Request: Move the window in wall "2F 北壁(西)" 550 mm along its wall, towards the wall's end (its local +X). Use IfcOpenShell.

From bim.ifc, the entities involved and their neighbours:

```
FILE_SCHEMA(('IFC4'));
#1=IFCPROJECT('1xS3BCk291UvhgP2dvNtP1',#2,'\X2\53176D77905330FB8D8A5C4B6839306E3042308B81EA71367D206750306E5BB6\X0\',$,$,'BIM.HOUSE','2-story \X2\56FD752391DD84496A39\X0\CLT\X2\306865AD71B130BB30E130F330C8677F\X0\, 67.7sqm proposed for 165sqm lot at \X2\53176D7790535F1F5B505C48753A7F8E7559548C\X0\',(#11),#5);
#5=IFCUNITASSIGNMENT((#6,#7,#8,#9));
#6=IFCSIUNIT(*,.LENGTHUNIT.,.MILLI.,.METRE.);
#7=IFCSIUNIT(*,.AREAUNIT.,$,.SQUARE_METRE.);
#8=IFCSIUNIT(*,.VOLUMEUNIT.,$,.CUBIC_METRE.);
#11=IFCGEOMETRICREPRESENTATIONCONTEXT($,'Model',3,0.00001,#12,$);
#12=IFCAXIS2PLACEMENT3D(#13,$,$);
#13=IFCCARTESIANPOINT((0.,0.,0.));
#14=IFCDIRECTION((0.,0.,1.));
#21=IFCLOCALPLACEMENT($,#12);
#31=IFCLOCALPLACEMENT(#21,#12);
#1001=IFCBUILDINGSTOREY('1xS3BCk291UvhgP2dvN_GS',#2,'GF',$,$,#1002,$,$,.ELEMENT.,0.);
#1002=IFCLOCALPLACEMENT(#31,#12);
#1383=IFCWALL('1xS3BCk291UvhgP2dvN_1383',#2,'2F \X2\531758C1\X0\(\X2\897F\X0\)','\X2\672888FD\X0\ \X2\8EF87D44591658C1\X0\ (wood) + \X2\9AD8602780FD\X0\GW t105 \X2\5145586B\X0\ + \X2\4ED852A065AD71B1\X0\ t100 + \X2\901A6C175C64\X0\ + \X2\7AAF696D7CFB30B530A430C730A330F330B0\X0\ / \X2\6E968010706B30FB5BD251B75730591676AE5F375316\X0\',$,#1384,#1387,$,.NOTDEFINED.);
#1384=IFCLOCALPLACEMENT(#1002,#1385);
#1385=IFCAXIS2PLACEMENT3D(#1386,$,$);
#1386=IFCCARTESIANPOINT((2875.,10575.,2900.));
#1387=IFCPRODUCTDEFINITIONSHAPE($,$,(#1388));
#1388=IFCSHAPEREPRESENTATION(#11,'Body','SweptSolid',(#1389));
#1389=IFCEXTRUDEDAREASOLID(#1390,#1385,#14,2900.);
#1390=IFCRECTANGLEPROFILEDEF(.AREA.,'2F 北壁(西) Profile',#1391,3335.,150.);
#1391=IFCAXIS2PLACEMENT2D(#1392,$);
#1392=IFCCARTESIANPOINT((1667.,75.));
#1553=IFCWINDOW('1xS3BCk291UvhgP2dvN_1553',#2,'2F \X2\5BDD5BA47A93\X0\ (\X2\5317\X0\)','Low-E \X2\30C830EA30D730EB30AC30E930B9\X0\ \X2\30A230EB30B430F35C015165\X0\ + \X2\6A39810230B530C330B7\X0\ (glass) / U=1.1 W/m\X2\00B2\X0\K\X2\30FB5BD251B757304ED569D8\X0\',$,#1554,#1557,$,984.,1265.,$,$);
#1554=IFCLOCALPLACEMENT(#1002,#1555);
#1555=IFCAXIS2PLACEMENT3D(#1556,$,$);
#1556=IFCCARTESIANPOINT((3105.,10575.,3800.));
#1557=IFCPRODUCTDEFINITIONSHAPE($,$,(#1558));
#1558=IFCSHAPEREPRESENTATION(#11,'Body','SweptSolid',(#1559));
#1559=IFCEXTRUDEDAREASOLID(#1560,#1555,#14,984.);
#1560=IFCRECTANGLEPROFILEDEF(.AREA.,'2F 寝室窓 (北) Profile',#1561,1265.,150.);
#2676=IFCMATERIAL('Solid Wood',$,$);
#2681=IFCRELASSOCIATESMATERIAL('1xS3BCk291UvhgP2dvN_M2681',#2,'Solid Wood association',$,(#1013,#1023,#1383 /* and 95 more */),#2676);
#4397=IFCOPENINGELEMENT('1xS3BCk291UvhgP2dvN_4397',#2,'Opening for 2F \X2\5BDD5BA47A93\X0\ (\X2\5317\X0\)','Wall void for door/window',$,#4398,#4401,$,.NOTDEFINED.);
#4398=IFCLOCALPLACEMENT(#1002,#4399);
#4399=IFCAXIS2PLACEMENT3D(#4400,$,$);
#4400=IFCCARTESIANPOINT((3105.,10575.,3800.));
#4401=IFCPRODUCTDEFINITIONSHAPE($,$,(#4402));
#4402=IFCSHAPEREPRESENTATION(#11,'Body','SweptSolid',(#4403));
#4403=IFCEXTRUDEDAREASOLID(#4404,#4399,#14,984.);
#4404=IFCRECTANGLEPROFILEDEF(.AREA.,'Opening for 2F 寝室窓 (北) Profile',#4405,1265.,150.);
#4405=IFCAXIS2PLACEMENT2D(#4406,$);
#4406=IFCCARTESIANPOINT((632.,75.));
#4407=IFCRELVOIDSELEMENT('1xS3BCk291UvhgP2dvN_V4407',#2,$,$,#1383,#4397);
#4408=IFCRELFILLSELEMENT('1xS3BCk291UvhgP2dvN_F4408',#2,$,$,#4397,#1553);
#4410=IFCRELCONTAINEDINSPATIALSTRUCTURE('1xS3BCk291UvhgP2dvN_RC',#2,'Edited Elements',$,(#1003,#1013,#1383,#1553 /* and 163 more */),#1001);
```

```python
import ifcopenshell
import ifcopenshell.api.geometry
import ifcopenshell.util.placement
import ifcopenshell.util.unit

model = ifcopenshell.open("bim.ifc")
unit_scale = ifcopenshell.util.unit.calculate_unit_scale(model)

window = model.by_guid("1xS3BCk291UvhgP2dvN_1553")
opening = window.FillsVoids[0].RelatingOpeningElement
wall = opening.VoidsElements[0].RelatingBuildingElement

wall_matrix = ifcopenshell.util.placement.get_local_placement(wall.ObjectPlacement)
shift = wall_matrix[:3, 0] * 0.55 / unit_scale
before = ifcopenshell.util.placement.get_local_placement(window.ObjectPlacement)[:3, 3].copy()

# The window is not placed relative to its opening, so move both.
for product in (opening, window):
    matrix = ifcopenshell.util.placement.get_local_placement(product.ObjectPlacement)
    matrix[:3, 3] += shift
    ifcopenshell.api.geometry.edit_object_placement(model, product=product, matrix=matrix, is_si=False)

after = ifcopenshell.util.placement.get_local_placement(window.ObjectPlacement)[:3, 3]
print("window moved by", (after - before).round(3) + 0.0)

model.write("bim-out.ifc")
```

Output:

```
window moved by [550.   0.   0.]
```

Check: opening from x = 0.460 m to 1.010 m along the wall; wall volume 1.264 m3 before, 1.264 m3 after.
